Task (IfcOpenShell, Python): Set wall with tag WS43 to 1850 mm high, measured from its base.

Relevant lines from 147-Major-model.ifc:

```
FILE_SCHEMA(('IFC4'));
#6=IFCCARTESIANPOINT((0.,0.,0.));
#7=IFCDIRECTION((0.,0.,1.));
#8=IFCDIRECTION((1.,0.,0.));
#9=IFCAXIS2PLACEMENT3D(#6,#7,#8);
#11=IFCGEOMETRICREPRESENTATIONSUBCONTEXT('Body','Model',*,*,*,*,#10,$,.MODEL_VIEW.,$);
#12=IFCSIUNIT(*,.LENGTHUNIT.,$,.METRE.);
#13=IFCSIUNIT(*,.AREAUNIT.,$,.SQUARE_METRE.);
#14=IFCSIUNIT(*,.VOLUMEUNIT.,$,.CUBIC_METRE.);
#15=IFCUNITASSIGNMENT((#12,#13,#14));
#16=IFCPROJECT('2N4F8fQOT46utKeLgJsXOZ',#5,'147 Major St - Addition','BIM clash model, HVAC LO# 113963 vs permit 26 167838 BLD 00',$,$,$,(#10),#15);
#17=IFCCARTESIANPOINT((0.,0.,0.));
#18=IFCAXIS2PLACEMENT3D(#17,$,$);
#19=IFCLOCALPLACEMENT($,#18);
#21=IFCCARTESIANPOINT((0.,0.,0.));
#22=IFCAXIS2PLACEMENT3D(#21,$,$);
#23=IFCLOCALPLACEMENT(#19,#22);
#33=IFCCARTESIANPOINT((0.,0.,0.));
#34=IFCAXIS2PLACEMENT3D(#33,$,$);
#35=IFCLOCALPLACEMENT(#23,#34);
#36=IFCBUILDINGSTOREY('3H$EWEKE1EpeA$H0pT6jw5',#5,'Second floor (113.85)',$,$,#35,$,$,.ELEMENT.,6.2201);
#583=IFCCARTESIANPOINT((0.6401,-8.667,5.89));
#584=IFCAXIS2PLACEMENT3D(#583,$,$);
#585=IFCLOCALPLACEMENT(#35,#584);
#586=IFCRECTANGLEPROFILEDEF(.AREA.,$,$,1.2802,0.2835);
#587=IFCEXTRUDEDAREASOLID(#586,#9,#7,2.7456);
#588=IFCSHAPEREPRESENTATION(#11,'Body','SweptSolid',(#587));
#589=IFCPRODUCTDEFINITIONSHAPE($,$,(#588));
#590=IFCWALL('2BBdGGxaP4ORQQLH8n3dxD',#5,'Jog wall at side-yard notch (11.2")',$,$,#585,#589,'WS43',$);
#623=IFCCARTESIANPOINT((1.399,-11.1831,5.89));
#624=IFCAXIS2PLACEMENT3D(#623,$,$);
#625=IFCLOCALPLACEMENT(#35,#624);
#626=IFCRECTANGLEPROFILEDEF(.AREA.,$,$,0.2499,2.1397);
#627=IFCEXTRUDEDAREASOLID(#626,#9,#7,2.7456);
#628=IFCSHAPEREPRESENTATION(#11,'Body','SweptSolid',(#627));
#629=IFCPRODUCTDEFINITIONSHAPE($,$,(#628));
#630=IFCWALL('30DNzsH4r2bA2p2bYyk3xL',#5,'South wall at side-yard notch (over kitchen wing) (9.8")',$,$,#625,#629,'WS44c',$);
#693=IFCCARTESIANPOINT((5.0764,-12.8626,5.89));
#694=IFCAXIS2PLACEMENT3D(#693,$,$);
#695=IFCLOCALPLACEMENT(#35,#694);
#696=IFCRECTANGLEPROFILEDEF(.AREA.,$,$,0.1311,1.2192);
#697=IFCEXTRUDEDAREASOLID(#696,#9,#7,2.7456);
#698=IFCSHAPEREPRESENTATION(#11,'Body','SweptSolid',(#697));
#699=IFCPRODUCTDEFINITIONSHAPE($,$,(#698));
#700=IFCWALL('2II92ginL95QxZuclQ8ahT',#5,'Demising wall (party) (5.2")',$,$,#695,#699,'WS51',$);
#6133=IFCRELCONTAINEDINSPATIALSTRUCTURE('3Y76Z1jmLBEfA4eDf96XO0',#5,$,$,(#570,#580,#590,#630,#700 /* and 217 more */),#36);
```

```python
import ifcopenshell
import ifcopenshell.geom
import ifcopenshell.util.representation
import ifcopenshell.util.shape

model = ifcopenshell.open("147-Major-model.ifc")
settings = ifcopenshell.geom.settings()


def volume(element):
    """Net volume in cubic metres, openings subtracted."""
    shape = ifcopenshell.geom.create_shape(settings, element)
    return ifcopenshell.util.shape.get_volume(shape.geometry)


wall = model.by_id(590)
before = volume(wall)

body = ifcopenshell.util.representation.get_representation(wall, "Model", "Body")
solid = body.Items[0]
old_height = solid.Depth
solid.Depth = 1.85
after = volume(wall)

print(f"height {old_height:g} -> {solid.Depth:g}, volume {before:.3f} -> {after:.3f} m3")

model.write("147-Major-model-out.ifc")
```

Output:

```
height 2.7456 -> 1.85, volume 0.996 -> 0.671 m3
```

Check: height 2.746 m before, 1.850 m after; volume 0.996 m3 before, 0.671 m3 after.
